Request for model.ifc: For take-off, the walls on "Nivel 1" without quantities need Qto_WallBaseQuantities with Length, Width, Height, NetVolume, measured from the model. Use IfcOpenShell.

First a look at what the model holds.

```python
import ifcopenshell
import ifcopenshell.util.element
import ifcopenshell.util.unit

model = ifcopenshell.open("model.ifc")
print(model.schema)
for unit_type in ("LENGTHUNIT", "AREAUNIT", "VOLUMEUNIT"):
    print(unit_type, ifcopenshell.util.unit.calculate_unit_scale(model, unit_type))
storey = next(s for s in model.by_type("IfcBuildingStorey") if s.Name == "Nivel 1")
walls = [e for e in ifcopenshell.util.element.get_decomposition(storey) if e.is_a("IfcWall")]
for e in sorted(walls, key=lambda e: e.id()):
    print(e.id(), e.is_a(), e.Name, list(ifcopenshell.util.element.get_psets(e, qtos_only=True)), sep=" | ")
```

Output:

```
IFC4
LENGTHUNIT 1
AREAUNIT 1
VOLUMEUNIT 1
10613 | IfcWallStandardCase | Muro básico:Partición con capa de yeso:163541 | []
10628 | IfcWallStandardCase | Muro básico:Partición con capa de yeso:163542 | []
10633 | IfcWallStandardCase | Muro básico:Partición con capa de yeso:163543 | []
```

```python
import ifcopenshell
import ifcopenshell.api.pset
import ifcopenshell.geom
import ifcopenshell.util.element
import ifcopenshell.util.shape
import ifcopenshell.util.unit

model = ifcopenshell.open("model.ifc")
unit_scale = ifcopenshell.util.unit.calculate_unit_scale(model)
volume_scale = ifcopenshell.util.unit.calculate_unit_scale(model, "VOLUMEUNIT")
settings = ifcopenshell.geom.settings()

storey = next(s for s in model.by_type("IfcBuildingStorey") if s.Name == "Nivel 1")
walls = [e for e in ifcopenshell.util.element.get_decomposition(storey) if e.is_a("IfcWall")]

for e in sorted(walls, key=lambda e: e.id()):
    if ifcopenshell.util.element.get_psets(e, qtos_only=True, should_inherit=False):
        continue
    # Geometry comes back in metres, in the element's own axes.
    shape = ifcopenshell.geom.create_shape(settings, e)
    values = {
        "Length": ifcopenshell.util.shape.get_x(shape.geometry) / unit_scale,
        "Width": ifcopenshell.util.shape.get_y(shape.geometry) / unit_scale,
        "Height": ifcopenshell.util.shape.get_z(shape.geometry) / unit_scale,
        "NetVolume": ifcopenshell.util.shape.get_volume(shape.geometry) / volume_scale,
    }
    qto = ifcopenshell.api.pset.add_qto(model, product=e, name="Qto_WallBaseQuantities")
    ifcopenshell.api.pset.edit_qto(model, qto=qto, properties=values)
    print(e.id(), {k: round(v, 3) for k, v in values.items()})

model.write("model_v2.ifc")
```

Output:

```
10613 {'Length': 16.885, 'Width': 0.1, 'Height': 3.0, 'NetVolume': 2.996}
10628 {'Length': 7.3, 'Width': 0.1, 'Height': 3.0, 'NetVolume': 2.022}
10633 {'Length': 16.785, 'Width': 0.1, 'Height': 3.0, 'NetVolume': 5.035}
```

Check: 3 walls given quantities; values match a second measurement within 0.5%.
